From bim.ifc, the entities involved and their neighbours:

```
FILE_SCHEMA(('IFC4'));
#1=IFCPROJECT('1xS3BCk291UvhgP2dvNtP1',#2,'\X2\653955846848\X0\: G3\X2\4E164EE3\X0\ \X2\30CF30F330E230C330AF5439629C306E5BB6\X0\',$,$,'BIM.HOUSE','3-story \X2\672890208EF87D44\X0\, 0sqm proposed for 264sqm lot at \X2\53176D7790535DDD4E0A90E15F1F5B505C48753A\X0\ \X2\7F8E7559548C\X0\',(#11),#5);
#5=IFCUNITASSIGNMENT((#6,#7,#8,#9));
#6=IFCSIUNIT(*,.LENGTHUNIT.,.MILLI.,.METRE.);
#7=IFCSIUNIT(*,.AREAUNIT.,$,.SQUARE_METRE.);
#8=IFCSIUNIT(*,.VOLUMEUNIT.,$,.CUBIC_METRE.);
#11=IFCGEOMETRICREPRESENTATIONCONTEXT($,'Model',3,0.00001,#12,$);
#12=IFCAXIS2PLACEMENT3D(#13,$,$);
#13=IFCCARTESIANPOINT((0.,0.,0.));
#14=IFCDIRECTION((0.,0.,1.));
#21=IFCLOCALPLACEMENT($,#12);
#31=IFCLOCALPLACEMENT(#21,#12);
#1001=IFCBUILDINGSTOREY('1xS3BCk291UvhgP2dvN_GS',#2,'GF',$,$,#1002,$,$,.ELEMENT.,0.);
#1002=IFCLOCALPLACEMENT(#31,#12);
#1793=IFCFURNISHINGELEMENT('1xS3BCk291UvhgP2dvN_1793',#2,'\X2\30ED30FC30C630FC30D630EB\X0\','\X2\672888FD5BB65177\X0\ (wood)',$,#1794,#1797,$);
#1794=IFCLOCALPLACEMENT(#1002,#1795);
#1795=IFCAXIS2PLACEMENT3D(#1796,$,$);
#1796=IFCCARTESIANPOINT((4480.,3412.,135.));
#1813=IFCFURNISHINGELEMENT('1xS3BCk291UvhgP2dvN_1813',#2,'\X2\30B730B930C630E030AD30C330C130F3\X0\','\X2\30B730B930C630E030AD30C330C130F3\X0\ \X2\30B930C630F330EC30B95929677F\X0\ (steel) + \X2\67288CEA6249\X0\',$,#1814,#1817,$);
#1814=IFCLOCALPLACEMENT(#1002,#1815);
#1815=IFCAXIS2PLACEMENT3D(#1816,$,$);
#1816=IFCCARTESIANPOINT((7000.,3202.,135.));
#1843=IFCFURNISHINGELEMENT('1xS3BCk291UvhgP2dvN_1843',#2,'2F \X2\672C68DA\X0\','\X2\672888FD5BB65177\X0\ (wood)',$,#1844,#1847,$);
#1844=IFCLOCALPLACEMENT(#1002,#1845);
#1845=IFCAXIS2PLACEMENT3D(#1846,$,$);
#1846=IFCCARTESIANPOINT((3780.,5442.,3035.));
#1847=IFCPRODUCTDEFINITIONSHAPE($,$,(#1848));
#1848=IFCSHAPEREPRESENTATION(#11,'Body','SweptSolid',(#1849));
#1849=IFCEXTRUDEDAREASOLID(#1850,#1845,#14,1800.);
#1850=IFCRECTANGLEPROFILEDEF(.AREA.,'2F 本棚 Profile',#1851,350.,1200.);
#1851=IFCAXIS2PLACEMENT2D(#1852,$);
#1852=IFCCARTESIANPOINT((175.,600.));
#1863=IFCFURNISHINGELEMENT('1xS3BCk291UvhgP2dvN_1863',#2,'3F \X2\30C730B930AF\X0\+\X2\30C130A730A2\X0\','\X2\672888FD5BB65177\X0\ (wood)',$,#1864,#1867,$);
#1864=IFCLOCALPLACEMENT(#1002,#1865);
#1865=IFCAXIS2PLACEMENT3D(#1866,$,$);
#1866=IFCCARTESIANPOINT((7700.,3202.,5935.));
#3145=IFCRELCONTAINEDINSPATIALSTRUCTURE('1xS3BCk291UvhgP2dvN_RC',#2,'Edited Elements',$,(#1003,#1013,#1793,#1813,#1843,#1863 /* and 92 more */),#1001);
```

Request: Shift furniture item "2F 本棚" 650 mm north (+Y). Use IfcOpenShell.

```python
import ifcopenshell
import ifcopenshell.api.geometry
import ifcopenshell.util.placement

model = ifcopenshell.open("bim.ifc")

item = model.by_guid("1xS3BCk291UvhgP2dvN_1843")
matrix = ifcopenshell.util.placement.get_local_placement(item.ObjectPlacement)
matrix[1, 3] += 650.0
ifcopenshell.api.geometry.edit_object_placement(model, product=item, matrix=matrix, is_si=False)

print(ifcopenshell.util.placement.get_local_placement(item.ObjectPlacement).round(3) + 0.0)

model.write("bim-out.ifc")
```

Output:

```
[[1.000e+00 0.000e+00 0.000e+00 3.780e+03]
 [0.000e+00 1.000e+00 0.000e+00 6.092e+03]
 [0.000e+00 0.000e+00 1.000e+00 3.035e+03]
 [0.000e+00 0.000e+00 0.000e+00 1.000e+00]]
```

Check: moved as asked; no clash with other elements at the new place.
